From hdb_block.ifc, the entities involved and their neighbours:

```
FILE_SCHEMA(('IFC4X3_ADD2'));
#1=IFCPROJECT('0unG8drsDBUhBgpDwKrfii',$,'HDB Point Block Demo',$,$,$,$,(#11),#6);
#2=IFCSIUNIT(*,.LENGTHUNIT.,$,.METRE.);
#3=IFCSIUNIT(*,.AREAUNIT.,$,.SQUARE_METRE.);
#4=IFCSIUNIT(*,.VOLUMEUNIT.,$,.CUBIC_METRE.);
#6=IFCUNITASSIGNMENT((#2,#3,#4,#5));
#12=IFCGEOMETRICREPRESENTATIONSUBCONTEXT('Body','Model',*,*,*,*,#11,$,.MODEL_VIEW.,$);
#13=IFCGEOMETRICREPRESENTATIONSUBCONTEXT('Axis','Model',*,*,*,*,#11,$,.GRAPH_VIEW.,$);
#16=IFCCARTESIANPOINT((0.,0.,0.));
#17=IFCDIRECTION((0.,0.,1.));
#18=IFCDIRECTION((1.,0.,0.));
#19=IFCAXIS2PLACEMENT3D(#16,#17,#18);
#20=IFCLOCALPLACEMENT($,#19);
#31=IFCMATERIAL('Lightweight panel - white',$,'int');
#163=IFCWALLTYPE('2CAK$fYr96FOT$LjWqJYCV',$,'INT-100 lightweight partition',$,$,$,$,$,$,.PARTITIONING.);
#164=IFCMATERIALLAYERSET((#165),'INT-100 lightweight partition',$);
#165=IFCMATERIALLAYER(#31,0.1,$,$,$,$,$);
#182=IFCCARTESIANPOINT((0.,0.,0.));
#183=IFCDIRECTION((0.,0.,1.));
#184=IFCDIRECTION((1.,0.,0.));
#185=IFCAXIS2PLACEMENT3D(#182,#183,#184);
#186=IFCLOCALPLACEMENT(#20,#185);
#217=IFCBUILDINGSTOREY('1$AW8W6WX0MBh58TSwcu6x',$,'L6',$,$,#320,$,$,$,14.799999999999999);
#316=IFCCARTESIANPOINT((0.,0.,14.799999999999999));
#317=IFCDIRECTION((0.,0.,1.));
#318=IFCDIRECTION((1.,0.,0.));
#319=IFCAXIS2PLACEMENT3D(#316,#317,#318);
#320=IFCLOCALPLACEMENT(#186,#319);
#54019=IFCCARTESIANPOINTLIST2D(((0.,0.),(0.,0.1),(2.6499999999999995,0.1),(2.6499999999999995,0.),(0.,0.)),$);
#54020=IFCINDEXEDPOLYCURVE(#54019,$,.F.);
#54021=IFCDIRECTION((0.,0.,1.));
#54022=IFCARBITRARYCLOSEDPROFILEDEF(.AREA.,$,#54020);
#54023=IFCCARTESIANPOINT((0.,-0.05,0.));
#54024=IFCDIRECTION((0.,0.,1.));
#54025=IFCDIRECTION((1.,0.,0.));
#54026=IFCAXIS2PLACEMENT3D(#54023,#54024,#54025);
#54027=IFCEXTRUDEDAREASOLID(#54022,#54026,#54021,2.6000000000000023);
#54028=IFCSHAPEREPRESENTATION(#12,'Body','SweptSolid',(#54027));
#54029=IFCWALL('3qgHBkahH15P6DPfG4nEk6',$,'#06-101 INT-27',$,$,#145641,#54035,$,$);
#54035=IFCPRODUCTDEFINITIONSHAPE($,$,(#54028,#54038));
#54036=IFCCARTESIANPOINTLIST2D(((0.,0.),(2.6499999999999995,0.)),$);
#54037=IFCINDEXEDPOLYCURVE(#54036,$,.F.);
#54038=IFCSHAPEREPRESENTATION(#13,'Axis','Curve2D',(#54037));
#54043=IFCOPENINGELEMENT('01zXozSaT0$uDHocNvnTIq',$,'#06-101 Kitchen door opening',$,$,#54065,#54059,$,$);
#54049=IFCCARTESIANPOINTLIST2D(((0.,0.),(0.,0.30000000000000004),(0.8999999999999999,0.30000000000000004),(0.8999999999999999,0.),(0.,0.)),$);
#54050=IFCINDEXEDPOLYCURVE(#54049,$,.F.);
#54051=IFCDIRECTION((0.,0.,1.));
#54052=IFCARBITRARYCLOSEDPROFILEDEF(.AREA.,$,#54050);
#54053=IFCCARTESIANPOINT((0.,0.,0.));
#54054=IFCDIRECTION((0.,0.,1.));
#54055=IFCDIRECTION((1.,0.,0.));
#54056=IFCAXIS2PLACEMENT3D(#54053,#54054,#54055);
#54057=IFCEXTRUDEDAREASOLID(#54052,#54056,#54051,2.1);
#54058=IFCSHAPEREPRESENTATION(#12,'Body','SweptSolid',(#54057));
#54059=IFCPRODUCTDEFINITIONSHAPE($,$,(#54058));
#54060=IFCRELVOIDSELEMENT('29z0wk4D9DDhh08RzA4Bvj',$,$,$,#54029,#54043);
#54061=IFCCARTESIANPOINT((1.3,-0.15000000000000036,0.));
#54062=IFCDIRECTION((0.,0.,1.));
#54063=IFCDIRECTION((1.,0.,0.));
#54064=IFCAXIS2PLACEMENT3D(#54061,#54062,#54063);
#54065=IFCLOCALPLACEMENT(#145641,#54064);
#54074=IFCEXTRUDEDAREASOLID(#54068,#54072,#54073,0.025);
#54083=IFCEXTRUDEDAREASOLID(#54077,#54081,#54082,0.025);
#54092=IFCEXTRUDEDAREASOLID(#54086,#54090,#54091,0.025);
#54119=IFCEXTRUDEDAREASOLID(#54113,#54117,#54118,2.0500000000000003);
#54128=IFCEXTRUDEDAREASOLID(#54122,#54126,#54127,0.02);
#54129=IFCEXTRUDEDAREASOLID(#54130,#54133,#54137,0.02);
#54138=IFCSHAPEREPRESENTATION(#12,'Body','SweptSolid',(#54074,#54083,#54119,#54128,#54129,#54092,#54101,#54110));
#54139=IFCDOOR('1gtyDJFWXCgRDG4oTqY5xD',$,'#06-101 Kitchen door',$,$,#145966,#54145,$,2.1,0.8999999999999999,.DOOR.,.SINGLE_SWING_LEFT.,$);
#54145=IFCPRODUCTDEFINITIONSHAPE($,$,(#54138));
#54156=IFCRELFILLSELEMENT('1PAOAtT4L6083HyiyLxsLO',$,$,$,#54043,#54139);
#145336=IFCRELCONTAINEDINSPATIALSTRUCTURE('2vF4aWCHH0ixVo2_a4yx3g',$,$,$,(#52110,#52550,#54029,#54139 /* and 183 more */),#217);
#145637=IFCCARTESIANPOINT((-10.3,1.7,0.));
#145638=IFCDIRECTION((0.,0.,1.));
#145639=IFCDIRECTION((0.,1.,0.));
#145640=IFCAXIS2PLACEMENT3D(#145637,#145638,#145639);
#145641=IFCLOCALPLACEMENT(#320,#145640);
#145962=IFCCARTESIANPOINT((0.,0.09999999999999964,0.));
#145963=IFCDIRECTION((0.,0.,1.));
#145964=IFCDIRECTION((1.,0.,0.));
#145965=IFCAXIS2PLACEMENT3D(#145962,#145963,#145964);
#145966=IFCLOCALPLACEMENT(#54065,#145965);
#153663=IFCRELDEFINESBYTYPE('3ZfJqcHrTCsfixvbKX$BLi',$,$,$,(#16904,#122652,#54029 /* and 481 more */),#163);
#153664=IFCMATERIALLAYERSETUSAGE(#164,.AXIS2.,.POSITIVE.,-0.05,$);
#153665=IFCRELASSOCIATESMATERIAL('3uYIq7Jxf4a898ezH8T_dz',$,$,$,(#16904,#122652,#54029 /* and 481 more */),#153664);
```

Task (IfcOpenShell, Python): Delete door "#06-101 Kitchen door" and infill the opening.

```python
import ifcopenshell
import ifcopenshell.api.feature
import ifcopenshell.api.root
import ifcopenshell.geom
import ifcopenshell.util.shape

model = ifcopenshell.open("hdb_block.ifc")
settings = ifcopenshell.geom.settings()


def volume(element):
    """Net volume in cubic metres, openings subtracted."""
    shape = ifcopenshell.geom.create_shape(settings, element)
    return ifcopenshell.util.shape.get_volume(shape.geometry)


door = model.by_id(54139)
opening = door.FillsVoids[0].RelatingOpeningElement
wall = opening.VoidsElements[0].RelatingBuildingElement
before = volume(wall)

ifcopenshell.api.root.remove_product(model, product=door)
ifcopenshell.api.feature.remove_feature(model, feature=opening)

after = volume(wall)

print(f"wall volume {before:.3f} -> {after:.3f} m3")

model.write("hdb_block_edited.ifc")
```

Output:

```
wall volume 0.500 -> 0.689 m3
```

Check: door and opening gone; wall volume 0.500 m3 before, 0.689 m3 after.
